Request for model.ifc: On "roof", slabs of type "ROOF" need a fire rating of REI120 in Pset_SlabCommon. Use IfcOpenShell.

First a look at what the model holds.

```python
import ifcopenshell
import ifcopenshell.util.element

model = ifcopenshell.open("model.ifc")
print(model.schema)
storey = next(s for s in model.by_type("IfcBuildingStorey") if s.Name == "roof")
slabs = [e for e in ifcopenshell.util.element.get_decomposition(storey) if e.is_a("IfcSlab")]
seen = {}
for e in slabs:
    element_type = ifcopenshell.util.element.get_type(e)
    key = (element_type.Name if element_type != e and element_type else None, ifcopenshell.util.element.get_pset(e, "Pset_SlabCommon", "FireRating"))
    seen[key] = seen.get(key, 0) + 1
for (name, value), count in sorted(seen.items(), key=str):
    print(count, "x", name, "|", value)
```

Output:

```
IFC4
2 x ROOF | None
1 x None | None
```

```python
import ifcopenshell
import ifcopenshell.api.pset
import ifcopenshell.util.element

model = ifcopenshell.open("model.ifc")

storey = next(s for s in model.by_type("IfcBuildingStorey") if s.Name == "roof")
slabs = [e for e in ifcopenshell.util.element.get_decomposition(storey) if e.is_a("IfcSlab")]

count = 0
for e in slabs:
    element_type = ifcopenshell.util.element.get_type(e)
    if element_type in (None, e) or element_type.Name != "ROOF":
        continue
    # add_pset returns the element's existing set when there is one.
    pset = ifcopenshell.api.pset.add_pset(model, product=e, name="Pset_SlabCommon")
    ifcopenshell.api.pset.edit_pset(model, pset=pset, properties={"FireRating": "REI120"})
    count += 1

print(count, "slabs updated")

model.write("model_updated.ifc")
```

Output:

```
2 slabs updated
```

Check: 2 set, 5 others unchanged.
